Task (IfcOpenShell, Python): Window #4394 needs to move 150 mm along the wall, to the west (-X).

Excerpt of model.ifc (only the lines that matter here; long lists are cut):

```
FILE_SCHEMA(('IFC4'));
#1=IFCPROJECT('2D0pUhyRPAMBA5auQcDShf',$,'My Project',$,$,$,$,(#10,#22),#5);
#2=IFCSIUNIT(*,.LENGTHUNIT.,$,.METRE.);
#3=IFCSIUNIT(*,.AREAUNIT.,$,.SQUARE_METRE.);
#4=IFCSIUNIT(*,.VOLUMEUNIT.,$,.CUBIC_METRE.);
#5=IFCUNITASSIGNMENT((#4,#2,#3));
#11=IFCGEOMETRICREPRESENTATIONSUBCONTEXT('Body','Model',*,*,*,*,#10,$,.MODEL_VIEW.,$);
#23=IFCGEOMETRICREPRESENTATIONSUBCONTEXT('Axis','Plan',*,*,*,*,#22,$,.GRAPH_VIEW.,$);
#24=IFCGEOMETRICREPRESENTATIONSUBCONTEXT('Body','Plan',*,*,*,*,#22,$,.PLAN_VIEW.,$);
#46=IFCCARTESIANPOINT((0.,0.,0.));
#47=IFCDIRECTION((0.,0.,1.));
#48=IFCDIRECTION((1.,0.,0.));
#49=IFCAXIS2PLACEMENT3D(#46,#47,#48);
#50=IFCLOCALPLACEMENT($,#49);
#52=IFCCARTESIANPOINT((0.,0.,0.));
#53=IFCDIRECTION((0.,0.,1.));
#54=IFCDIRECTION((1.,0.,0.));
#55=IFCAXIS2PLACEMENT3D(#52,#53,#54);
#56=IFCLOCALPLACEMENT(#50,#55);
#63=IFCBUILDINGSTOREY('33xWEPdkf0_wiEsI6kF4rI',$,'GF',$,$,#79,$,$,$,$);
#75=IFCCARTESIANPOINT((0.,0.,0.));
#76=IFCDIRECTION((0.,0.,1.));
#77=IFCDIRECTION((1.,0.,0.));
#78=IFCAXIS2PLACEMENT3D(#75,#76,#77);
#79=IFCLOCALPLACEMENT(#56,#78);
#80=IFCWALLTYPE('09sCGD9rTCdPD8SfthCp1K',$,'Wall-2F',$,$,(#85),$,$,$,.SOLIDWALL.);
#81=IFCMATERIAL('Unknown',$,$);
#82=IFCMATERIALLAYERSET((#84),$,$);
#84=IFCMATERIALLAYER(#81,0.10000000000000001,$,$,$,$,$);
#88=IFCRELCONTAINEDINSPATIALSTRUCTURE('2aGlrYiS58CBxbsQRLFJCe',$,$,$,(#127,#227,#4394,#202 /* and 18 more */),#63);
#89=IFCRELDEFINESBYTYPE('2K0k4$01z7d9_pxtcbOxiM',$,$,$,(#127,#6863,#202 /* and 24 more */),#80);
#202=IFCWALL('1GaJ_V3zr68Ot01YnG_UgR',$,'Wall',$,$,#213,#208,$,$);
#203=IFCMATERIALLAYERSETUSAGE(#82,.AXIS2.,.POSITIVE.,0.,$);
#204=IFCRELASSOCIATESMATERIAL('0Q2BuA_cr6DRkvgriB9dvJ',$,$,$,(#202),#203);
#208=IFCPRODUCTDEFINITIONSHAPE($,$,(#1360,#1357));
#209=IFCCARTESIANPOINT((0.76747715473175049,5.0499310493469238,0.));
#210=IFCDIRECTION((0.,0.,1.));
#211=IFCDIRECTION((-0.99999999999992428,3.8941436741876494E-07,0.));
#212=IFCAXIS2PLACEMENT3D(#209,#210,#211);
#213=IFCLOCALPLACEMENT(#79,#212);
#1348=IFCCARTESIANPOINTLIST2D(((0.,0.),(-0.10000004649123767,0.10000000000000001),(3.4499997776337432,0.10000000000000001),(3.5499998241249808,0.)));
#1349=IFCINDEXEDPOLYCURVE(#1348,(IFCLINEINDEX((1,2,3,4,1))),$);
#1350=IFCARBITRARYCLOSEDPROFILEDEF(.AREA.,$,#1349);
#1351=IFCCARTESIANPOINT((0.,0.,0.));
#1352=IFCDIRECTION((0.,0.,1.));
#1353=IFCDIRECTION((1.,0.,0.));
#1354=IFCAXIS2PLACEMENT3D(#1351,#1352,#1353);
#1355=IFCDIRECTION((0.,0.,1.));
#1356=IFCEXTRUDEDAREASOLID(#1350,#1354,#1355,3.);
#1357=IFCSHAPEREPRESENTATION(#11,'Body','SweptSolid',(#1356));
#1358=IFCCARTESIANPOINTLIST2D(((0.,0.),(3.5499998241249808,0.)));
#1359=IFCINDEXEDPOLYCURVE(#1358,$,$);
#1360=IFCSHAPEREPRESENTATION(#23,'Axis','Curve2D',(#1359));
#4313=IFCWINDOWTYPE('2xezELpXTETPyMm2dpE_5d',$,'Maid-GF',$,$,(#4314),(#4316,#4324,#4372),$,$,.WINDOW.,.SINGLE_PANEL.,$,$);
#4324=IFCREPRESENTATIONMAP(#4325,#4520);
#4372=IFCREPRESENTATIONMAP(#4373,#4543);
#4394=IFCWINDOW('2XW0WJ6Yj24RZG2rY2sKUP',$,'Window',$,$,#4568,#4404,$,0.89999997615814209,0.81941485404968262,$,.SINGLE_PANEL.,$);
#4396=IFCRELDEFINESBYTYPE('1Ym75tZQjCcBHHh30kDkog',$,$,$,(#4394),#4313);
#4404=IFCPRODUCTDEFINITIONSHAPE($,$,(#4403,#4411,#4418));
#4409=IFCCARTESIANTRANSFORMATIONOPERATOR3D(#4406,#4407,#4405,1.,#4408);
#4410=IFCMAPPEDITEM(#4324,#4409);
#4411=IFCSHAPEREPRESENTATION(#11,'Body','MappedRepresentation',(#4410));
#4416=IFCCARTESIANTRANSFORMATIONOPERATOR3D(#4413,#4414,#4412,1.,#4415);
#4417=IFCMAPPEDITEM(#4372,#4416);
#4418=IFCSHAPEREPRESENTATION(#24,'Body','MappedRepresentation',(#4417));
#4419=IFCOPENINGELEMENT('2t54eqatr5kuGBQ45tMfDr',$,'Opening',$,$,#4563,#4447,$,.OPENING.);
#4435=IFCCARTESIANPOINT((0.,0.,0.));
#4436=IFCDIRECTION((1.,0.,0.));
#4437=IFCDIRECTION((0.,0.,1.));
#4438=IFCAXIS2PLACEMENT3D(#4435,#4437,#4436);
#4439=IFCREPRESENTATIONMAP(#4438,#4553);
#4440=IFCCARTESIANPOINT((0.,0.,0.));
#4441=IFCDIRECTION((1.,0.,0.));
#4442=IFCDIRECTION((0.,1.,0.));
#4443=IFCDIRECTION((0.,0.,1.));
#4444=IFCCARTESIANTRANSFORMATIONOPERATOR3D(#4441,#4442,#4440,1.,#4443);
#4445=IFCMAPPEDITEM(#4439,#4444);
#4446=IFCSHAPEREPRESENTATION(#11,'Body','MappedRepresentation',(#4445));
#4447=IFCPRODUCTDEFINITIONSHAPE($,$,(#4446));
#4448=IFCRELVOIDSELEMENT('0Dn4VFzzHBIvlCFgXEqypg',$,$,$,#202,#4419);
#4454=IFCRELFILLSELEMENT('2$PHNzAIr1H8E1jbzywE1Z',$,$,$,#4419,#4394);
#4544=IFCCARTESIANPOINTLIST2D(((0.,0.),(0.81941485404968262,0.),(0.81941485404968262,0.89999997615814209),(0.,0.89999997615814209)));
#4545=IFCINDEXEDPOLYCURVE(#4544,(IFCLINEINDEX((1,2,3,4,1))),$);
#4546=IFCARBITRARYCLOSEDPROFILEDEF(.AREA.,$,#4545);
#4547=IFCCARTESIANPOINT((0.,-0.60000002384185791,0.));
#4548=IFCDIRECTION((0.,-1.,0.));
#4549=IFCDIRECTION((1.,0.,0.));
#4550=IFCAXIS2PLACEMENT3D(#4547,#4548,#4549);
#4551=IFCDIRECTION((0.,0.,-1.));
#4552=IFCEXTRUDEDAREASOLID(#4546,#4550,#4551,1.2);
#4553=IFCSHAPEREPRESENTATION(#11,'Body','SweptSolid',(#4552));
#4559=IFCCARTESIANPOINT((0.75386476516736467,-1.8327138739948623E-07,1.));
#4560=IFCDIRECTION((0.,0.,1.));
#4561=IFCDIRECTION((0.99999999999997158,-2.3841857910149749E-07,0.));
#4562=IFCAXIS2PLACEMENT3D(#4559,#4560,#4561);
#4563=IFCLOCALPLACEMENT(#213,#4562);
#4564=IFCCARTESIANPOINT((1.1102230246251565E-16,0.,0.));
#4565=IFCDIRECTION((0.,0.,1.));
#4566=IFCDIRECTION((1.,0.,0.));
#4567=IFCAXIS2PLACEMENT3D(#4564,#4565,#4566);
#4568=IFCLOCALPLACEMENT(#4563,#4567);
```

```python
import ifcopenshell
import ifcopenshell.api.geometry
import ifcopenshell.util.placement
import ifcopenshell.util.unit

model = ifcopenshell.open("model.ifc")
unit_scale = ifcopenshell.util.unit.calculate_unit_scale(model)

window = model.by_guid("2XW0WJ6Yj24RZG2rY2sKUP")
opening = window.FillsVoids[0].RelatingOpeningElement
wall = opening.VoidsElements[0].RelatingBuildingElement

wall_matrix = ifcopenshell.util.placement.get_local_placement(wall.ObjectPlacement)
shift = wall_matrix[:3, 0] * 0.15 / unit_scale
before = ifcopenshell.util.placement.get_local_placement(window.ObjectPlacement)[:3, 3].copy()

# The window is placed relative to its opening, so it follows when the opening moves.
matrix = ifcopenshell.util.placement.get_local_placement(opening.ObjectPlacement)
matrix[:3, 3] += shift
ifcopenshell.api.geometry.edit_object_placement(
    model, product=opening, matrix=matrix, is_si=False, should_transform_children=True
)

after = ifcopenshell.util.placement.get_local_placement(window.ObjectPlacement)[:3, 3]
print("window moved by", (after - before).round(3) + 0.0)

model.write("model_v2.ifc")
```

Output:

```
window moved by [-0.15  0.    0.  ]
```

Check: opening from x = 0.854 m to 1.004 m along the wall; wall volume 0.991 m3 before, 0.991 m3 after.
